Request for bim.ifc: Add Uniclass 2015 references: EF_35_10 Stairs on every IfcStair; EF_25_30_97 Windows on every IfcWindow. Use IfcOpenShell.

First a look at what the model holds.

```python
import ifcopenshell

model = ifcopenshell.open("bim.ifc")
print(model.schema)
print("classifications:", [c.Name for c in model.by_type("IfcClassification")])
for ifc_class in ("IfcDoor", "IfcRoof", "IfcStair", "IfcWall", "IfcWindow"):
    print(ifc_class, len(model.by_type(ifc_class)))
```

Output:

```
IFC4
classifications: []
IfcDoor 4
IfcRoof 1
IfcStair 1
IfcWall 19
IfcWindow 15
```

```python
import ifcopenshell
import ifcopenshell.api.classification

model = ifcopenshell.open("bim.ifc")

system = ifcopenshell.api.classification.add_classification(model, classification="Uniclass 2015")

codes = {
    "IfcStair": ("EF_35_10", "Stairs"),
    "IfcWindow": ("EF_25_30_97", "Windows"),
}
for ifc_class, (code, name) in codes.items():
    products = model.by_type(ifc_class)
    ifcopenshell.api.classification.add_reference(
        model, products=products, classification=system, identification=code, name=name
    )
    print(code, len(products))

model.write("bim-out.ifc")
```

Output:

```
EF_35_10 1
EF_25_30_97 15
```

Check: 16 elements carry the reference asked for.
